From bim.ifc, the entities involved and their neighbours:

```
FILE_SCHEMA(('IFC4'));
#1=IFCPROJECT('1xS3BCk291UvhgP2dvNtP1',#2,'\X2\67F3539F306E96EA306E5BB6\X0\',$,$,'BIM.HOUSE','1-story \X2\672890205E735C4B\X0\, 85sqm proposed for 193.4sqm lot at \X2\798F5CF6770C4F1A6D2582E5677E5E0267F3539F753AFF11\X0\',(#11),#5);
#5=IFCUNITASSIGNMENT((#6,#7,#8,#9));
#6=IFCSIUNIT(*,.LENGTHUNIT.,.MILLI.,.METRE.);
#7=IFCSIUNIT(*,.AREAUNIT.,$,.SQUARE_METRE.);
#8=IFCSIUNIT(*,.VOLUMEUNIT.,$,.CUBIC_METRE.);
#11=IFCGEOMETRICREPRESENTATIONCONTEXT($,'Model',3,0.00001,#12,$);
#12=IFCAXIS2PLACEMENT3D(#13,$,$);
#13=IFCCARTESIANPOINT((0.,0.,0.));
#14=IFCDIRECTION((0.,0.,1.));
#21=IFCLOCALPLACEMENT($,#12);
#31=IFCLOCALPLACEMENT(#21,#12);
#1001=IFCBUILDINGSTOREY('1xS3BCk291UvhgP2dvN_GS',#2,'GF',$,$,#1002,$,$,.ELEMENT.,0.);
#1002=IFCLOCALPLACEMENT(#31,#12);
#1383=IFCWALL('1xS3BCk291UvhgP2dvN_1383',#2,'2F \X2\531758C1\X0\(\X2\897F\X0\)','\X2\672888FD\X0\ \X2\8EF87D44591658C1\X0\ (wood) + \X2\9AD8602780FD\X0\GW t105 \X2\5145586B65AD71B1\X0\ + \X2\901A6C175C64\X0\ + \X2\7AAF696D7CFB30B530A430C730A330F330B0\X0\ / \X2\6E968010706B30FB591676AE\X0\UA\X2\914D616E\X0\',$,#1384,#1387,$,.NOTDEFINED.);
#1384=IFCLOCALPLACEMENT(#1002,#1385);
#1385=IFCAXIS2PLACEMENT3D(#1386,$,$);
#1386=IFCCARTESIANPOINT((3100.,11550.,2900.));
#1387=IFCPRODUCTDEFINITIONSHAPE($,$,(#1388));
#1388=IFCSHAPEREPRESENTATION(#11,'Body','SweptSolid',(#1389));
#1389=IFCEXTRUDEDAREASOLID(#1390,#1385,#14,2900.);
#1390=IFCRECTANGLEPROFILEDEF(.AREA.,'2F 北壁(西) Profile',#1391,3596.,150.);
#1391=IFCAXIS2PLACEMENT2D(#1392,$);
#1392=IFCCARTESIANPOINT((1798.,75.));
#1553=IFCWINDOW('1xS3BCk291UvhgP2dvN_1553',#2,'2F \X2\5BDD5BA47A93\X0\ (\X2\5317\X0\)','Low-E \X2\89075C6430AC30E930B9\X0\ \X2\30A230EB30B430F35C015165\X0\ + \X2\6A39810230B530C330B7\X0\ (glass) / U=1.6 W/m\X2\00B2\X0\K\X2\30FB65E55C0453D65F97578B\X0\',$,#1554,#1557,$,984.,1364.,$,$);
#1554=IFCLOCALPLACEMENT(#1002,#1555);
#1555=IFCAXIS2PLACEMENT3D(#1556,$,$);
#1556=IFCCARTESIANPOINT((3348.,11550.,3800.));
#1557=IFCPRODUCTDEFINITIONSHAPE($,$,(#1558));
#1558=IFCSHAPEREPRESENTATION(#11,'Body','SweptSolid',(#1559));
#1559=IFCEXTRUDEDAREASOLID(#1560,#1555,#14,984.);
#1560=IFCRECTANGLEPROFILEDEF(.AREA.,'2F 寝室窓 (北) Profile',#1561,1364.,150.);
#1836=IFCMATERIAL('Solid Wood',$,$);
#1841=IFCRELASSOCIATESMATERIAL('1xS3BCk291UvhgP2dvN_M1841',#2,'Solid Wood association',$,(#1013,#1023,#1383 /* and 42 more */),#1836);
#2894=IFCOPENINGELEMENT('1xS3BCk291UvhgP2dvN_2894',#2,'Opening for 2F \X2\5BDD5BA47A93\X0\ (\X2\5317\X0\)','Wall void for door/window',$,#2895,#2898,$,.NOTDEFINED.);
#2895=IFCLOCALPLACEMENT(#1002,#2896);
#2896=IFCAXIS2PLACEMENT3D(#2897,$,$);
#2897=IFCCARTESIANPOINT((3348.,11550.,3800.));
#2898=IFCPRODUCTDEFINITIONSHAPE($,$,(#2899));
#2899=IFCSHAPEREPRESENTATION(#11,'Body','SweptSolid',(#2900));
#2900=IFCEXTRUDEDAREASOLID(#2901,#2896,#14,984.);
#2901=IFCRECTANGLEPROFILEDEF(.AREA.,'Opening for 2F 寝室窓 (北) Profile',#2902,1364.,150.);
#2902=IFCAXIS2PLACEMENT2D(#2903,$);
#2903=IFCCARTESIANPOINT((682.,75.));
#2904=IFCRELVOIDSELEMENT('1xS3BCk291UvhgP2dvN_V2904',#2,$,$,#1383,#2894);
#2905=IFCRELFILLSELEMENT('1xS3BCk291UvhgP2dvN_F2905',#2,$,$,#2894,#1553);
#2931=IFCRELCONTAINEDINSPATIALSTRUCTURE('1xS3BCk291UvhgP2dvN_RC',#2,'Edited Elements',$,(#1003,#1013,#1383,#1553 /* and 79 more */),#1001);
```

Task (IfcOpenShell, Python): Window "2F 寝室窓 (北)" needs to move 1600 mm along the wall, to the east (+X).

```python
import ifcopenshell
import ifcopenshell.api.geometry
import ifcopenshell.util.placement

model = ifcopenshell.open("bim.ifc")

window = model.by_id(1553)
opening = window.FillsVoids[0].RelatingOpeningElement
wall = opening.VoidsElements[0].RelatingBuildingElement

wall_matrix = ifcopenshell.util.placement.get_local_placement(wall.ObjectPlacement)
shift = wall_matrix[:3, 0] * 1600.0
before = ifcopenshell.util.placement.get_local_placement(window.ObjectPlacement)[:3, 3].copy()

# The window is not placed relative to its opening, so move both.
for product in (opening, window):
    matrix = ifcopenshell.util.placement.get_local_placement(product.ObjectPlacement)
    matrix[:3, 3] += shift
    ifcopenshell.api.geometry.edit_object_placement(model, product=product, matrix=matrix, is_si=False)

after = ifcopenshell.util.placement.get_local_placement(window.ObjectPlacement)[:3, 3]
print("window moved by", (after - before).round(3) + 0.0)

model.write("bim_rev.ifc")
```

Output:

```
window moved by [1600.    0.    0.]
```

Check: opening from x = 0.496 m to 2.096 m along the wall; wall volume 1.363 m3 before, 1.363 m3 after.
